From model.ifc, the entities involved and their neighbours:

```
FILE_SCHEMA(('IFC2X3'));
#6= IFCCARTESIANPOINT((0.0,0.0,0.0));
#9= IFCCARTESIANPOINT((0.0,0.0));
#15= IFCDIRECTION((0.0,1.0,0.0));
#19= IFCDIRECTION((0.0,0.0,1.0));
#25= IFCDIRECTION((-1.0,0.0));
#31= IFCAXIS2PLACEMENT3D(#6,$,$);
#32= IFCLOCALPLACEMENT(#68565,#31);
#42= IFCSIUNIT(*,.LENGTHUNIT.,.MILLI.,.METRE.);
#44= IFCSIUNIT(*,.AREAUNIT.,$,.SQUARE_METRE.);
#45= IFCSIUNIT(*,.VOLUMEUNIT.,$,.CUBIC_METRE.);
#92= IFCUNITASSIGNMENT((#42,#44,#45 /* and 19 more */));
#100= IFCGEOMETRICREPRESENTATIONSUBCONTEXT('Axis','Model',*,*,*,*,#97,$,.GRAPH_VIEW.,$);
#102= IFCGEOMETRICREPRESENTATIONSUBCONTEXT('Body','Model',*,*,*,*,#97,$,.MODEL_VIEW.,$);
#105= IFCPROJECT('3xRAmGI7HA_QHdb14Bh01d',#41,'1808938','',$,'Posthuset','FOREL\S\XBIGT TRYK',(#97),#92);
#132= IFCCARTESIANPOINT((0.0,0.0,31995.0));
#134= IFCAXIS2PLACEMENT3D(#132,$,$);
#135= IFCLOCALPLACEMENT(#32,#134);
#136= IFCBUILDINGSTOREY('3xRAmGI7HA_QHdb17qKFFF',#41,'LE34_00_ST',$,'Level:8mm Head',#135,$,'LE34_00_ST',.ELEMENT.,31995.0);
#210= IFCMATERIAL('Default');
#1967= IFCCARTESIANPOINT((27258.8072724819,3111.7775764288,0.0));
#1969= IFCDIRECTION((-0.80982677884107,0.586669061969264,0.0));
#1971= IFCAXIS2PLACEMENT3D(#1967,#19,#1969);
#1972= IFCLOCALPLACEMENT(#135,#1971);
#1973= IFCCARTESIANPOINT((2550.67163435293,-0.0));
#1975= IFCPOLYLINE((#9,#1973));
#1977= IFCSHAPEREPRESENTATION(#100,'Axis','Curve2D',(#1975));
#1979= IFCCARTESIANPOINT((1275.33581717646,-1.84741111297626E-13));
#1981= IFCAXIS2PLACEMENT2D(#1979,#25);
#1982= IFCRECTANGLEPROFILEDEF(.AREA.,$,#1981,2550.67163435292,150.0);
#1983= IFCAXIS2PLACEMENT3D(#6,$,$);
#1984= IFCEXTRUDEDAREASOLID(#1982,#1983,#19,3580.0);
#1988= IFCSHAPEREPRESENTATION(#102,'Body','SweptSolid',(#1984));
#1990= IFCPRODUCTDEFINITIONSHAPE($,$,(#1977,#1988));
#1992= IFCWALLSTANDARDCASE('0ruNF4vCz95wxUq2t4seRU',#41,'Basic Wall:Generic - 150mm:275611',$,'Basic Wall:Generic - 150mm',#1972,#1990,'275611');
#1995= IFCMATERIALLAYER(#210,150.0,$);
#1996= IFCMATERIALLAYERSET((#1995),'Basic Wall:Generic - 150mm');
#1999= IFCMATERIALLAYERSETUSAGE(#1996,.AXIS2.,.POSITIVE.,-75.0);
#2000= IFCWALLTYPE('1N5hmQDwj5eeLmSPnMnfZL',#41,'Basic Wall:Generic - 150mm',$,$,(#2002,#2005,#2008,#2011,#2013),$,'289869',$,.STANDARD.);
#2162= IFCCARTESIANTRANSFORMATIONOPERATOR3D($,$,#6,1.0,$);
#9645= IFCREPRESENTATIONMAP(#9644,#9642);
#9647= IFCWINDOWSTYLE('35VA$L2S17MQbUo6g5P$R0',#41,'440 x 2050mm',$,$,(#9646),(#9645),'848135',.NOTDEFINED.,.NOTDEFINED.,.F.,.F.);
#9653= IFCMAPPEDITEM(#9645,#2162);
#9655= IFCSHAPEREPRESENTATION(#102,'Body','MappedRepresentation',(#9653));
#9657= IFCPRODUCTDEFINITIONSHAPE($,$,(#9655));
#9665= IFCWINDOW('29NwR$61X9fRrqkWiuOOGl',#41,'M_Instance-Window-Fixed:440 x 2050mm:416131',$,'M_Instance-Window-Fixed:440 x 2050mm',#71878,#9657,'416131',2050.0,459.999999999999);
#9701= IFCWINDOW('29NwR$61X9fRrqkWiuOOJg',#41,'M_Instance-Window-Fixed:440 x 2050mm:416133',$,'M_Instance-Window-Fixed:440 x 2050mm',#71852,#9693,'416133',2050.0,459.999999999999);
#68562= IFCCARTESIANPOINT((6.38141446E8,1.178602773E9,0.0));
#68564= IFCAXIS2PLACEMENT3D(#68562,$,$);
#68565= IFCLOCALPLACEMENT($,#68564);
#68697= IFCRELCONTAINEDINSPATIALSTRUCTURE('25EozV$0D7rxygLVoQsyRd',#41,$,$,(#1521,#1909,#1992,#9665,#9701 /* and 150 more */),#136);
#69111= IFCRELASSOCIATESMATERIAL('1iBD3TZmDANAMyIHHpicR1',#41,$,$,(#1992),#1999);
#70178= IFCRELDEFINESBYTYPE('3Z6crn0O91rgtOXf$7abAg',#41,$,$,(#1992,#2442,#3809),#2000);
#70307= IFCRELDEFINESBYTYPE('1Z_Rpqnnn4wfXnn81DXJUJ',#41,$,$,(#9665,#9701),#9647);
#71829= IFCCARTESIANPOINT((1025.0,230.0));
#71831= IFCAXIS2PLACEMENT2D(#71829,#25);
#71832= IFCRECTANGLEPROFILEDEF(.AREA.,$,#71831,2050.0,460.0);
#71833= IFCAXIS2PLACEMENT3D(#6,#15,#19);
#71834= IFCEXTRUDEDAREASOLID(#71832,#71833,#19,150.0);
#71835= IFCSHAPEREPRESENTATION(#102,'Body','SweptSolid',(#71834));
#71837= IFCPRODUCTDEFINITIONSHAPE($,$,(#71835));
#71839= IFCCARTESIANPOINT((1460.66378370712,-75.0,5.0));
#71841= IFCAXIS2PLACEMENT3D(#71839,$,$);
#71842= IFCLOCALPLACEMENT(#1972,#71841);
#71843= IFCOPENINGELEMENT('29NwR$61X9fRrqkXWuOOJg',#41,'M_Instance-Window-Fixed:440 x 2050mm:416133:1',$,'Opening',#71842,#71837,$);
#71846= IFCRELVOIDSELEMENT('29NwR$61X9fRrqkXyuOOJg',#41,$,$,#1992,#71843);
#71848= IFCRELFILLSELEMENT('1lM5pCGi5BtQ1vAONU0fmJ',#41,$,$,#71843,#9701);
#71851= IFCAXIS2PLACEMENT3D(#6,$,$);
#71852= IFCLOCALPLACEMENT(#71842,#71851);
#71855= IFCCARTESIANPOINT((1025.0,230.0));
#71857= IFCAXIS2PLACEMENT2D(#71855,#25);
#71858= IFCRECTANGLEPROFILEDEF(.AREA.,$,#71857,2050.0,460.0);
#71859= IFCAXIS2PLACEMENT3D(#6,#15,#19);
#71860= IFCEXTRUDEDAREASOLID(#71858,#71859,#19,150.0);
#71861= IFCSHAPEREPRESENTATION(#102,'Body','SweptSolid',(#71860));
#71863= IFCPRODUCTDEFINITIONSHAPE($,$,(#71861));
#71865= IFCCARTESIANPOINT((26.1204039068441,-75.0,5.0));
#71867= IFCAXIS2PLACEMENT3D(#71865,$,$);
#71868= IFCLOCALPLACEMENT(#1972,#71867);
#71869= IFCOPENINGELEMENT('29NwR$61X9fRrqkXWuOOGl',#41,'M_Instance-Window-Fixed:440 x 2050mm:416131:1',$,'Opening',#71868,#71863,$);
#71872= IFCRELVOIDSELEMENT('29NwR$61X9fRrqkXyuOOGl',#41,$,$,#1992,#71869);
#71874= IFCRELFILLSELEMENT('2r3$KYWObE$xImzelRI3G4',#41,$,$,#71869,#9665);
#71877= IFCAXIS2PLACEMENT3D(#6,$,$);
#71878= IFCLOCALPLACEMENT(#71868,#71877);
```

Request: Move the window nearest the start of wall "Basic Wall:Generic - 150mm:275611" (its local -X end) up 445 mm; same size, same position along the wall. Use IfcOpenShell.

```python
import numpy as np
import ifcopenshell
import ifcopenshell.api.geometry
import ifcopenshell.util.placement
import ifcopenshell.util.unit

model = ifcopenshell.open("model.ifc")
unit_scale = ifcopenshell.util.unit.calculate_unit_scale(model)

window = model.by_id(9665)
opening = window.FillsVoids[0].RelatingOpeningElement
dz = 0.445 / unit_scale

shift = np.array([0.0, 0.0, dz])
# The window is placed relative to its opening, so it follows when the opening moves.
matrix = ifcopenshell.util.placement.get_local_placement(opening.ObjectPlacement)
matrix[:3, 3] += shift
ifcopenshell.api.geometry.edit_object_placement(
    model, product=opening, matrix=matrix, is_si=False, should_transform_children=True
)

print(f"moved by {dz * unit_scale:+.3f} m")

model.write("model_updated.ifc")
```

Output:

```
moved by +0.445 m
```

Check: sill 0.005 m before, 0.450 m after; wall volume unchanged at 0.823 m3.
